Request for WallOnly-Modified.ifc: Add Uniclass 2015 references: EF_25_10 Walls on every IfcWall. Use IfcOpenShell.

First a look at what the model holds.

```python
import ifcopenshell

model = ifcopenshell.open("WallOnly-Modified.ifc")
print(model.schema)
print("classifications:", [c.Name for c in model.by_type("IfcClassification")])
for ifc_class in ("IfcDoor", "IfcRoof", "IfcStair", "IfcWall", "IfcWindow"):
    print(ifc_class, len(model.by_type(ifc_class)))
```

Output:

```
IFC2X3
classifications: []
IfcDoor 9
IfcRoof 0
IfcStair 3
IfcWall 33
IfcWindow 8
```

```python
import ifcopenshell
import ifcopenshell.api.classification

model = ifcopenshell.open("WallOnly-Modified.ifc")

# IFC2X3 requires Source and Edition and has no link from the project to the system.
system = model.create_entity("IfcClassification", Source="NBS", Edition="2015", Name="Uniclass 2015")

codes = {
    "IfcWall": ("EF_25_10", "Walls"),
}
for ifc_class, (code, name) in codes.items():
    products = model.by_type(ifc_class)
    ifcopenshell.api.classification.add_reference(
        model, products=products, classification=system, identification=code, name=name
    )
    print(code, len(products))

model.write("WallOnly-Modified_edited.ifc")
```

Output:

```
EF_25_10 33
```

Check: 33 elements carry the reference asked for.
